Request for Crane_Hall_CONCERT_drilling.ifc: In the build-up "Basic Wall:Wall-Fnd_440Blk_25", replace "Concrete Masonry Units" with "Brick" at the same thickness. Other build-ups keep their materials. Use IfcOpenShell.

First a look at what the model holds.

```python
import ifcopenshell
import ifcopenshell.util.element

model = ifcopenshell.open("Crane_Hall_CONCERT_drilling.ifc")
print(model.schema)
for layer_set in model.by_type("IfcMaterialLayerSet"):
    if layer_set.LayerSetName == "Basic Wall:Wall-Fnd_440Blk_25":
        for layer in layer_set.MaterialLayers:
            print(layer.id(), layer.Material and layer.Material.Name, layer.LayerThickness, sep=" | ")
        print(len(ifcopenshell.util.element.get_elements_by_material(model, layer_set)), "elements and types use it")
print(sorted(m.Name for m in model.by_type("IfcMaterial") if m.Name)[:60])
```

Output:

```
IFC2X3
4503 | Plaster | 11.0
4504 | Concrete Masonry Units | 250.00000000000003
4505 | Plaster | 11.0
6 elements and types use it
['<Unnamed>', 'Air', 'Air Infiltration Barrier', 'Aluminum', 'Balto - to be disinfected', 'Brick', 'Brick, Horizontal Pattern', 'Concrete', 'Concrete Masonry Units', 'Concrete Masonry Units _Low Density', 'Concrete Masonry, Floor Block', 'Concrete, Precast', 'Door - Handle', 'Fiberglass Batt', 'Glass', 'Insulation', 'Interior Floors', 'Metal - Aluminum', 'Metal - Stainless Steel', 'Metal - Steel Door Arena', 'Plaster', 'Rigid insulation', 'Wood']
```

```python
import ifcopenshell
import ifcopenshell.api.material

model = ifcopenshell.open("Crane_Hall_CONCERT_drilling.ifc")

layer_set = next(s for s in model.by_type("IfcMaterialLayerSet") if s.LayerSetName == "Basic Wall:Wall-Fnd_440Blk_25")
layer = next(l for l in layer_set.MaterialLayers if l.Material and l.Material.Name == "Concrete Masonry Units")
material = next(m for m in model.by_type("IfcMaterial") if m.Name == "Brick")

# Point this one layer at the other material; renaming the old one would change it everywhere.
ifcopenshell.api.material.edit_layer(model, layer=layer, attributes={}, material=material)

print([l.Material.Name if l.Material else None for l in layer_set.MaterialLayers])

model.write("Crane_Hall_CONCERT_drilling-out.ifc")
```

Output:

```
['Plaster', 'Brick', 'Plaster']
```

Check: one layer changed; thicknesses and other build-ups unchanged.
